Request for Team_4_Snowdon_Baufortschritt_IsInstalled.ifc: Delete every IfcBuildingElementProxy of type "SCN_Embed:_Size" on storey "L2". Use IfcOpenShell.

First a look at what the model holds.

```python
import ifcopenshell
import ifcopenshell.util.element

model = ifcopenshell.open("Team_4_Snowdon_Baufortschritt_IsInstalled.ifc")
print(model.schema)
storey = next(s for s in model.by_type("IfcBuildingStorey") if s.Name == "L2")
proxies = [e for e in ifcopenshell.util.element.get_decomposition(storey) if e.is_a("IfcBuildingElementProxy")]
seen = {}
for e in proxies:
    element_type = ifcopenshell.util.element.get_type(e)
    name = element_type.Name if element_type not in (None, e) else None
    seen[name] = seen.get(name, 0) + 1
for name, count in sorted(seen.items(), key=str):
    print(count, "x", name)
```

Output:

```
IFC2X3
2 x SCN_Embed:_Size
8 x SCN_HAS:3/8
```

```python
import ifcopenshell
import ifcopenshell.api.root
import ifcopenshell.util.element

model = ifcopenshell.open("Team_4_Snowdon_Baufortschritt_IsInstalled.ifc")

storey = next(s for s in model.by_type("IfcBuildingStorey") if s.Name == "L2")
proxies = [e for e in ifcopenshell.util.element.get_decomposition(storey) if e.is_a("IfcBuildingElementProxy")]
targets = [e for e in proxies if (t := ifcopenshell.util.element.get_type(e)) not in (None, e) and t.Name == "SCN_Embed:_Size"]

for e in targets:
    ifcopenshell.api.root.remove_product(model, product=e)
print(len(targets), "removed")

model.write("Team_4_Snowdon_Baufortschritt_IsInstalled_updated.ifc")
```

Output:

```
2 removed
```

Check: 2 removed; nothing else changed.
